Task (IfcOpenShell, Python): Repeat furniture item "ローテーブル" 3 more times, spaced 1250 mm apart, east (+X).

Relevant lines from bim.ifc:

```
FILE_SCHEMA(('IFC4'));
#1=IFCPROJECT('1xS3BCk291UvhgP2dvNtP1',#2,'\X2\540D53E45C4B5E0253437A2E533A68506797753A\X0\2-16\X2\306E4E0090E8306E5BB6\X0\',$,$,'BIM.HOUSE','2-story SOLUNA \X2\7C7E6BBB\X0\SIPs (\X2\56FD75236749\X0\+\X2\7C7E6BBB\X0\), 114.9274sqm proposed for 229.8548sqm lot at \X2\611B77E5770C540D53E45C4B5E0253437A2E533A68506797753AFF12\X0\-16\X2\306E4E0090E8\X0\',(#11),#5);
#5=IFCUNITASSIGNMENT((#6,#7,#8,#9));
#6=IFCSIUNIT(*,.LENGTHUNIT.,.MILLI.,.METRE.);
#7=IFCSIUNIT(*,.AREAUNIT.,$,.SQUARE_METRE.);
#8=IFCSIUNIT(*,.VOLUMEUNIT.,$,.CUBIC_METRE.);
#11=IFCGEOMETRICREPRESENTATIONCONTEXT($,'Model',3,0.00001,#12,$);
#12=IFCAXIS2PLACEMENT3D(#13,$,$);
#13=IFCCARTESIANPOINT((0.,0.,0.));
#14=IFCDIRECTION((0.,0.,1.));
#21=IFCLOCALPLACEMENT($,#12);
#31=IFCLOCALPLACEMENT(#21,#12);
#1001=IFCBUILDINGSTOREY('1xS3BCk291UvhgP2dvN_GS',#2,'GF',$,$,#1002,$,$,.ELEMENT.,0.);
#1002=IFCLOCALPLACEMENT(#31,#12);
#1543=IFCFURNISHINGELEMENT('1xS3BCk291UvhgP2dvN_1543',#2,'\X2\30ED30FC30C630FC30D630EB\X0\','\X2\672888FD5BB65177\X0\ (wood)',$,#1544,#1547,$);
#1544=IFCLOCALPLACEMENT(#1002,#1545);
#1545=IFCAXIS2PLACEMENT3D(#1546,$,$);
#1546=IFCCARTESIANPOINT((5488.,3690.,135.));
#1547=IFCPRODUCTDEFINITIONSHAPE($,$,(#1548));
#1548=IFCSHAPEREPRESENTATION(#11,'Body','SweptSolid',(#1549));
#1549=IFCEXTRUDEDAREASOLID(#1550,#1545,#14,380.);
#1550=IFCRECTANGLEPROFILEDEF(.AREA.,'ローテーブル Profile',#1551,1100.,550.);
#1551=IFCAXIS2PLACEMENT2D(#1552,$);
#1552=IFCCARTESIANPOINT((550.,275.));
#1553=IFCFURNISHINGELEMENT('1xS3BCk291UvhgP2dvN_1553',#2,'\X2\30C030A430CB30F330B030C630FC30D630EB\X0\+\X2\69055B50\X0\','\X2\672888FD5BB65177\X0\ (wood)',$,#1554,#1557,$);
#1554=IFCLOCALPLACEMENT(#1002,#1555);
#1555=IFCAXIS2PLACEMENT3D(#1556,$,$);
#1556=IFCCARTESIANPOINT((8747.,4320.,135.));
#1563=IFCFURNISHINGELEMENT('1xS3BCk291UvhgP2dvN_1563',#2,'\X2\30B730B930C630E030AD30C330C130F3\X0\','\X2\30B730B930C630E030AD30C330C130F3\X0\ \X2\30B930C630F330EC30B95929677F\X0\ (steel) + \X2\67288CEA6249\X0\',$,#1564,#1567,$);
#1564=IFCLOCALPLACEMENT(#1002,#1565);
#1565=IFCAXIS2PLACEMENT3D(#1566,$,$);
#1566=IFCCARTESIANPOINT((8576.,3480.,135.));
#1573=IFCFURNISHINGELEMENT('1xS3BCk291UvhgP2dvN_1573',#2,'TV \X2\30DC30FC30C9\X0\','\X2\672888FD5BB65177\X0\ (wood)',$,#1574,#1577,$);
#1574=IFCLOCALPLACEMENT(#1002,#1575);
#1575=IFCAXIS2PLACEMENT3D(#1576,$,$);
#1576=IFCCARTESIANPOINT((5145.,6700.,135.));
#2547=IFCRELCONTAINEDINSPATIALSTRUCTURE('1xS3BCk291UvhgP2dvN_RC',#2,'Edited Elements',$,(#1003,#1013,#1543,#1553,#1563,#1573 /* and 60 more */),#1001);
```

```python
import numpy as np
import ifcopenshell
import ifcopenshell.api.geometry
import ifcopenshell.api.root
import ifcopenshell.util.element
import ifcopenshell.util.placement

model = ifcopenshell.open("bim.ifc")


def reuse_history(source, copy):
    """copy_class also copies each property set's owner history, people and application; keep the originals."""
    for rel in copy.IsDefinedBy:
        if rel.is_a("IfcRelDefinesByProperties") and (history := rel.RelatingPropertyDefinition.OwnerHistory):
            rel.RelatingPropertyDefinition.OwnerHistory = source.OwnerHistory
            ifcopenshell.util.element.remove_deep2(model, history)


source = model.by_guid("1xS3BCk291UvhgP2dvN_1543")
base = ifcopenshell.util.placement.get_local_placement(source.ObjectPlacement)
step = np.array([1.0, 0.0, 0.0]) * 1250.0

for i in range(1, 4):
    copy = ifcopenshell.api.root.copy_class(model, product=source)
    copy.Representation = ifcopenshell.util.element.copy_deep(
        model, source.Representation, exclude=["IfcGeometricRepresentationContext", "IfcRepresentationMap"]
    )
    reuse_history(source, copy)
    matrix = base.copy()
    matrix[:3, 3] += i * step
    print("added at", matrix[:3, 3].round(3) + 0.0)
    ifcopenshell.api.geometry.edit_object_placement(model, product=copy, matrix=matrix, is_si=False)

model.write("bim_rev.ifc")
```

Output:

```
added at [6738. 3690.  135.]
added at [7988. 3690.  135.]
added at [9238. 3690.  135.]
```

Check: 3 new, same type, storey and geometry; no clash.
